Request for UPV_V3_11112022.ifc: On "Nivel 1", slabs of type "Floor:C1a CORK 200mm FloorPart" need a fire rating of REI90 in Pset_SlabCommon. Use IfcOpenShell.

First a look at what the model holds.

```python
import ifcopenshell
import ifcopenshell.util.element

model = ifcopenshell.open("UPV_V3_11112022.ifc")
print(model.schema)
storey = next(s for s in model.by_type("IfcBuildingStorey") if s.Name == "Nivel 1")
slabs = [e for e in ifcopenshell.util.element.get_decomposition(storey) if e.is_a("IfcSlab")]
seen = {}
for e in slabs:
    element_type = ifcopenshell.util.element.get_type(e)
    key = (element_type.Name if element_type != e and element_type else None, ifcopenshell.util.element.get_pset(e, "Pset_SlabCommon", "FireRating"))
    seen[key] = seen.get(key, 0) + 1
for (name, value), count in sorted(seen.items(), key=str):
    print(count, "x", name, "|", value)
```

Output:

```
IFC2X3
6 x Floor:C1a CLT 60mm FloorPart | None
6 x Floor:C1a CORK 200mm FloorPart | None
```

```python
import ifcopenshell
import ifcopenshell.api.pset
import ifcopenshell.util.element

model = ifcopenshell.open("UPV_V3_11112022.ifc")

storey = next(s for s in model.by_type("IfcBuildingStorey") if s.Name == "Nivel 1")
slabs = [e for e in ifcopenshell.util.element.get_decomposition(storey) if e.is_a("IfcSlab")]

count = 0
for e in slabs:
    element_type = ifcopenshell.util.element.get_type(e)
    if element_type in (None, e) or element_type.Name != "Floor:C1a CORK 200mm FloorPart":
        continue
    # add_pset returns the element's existing set when there is one.
    pset = ifcopenshell.api.pset.add_pset(model, product=e, name="Pset_SlabCommon")
    ifcopenshell.api.pset.edit_pset(model, pset=pset, properties={"FireRating": "REI90"})
    count += 1

print(count, "slabs updated")

model.write("UPV_V3_11112022_v2.ifc")
```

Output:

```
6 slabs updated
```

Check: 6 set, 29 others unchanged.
